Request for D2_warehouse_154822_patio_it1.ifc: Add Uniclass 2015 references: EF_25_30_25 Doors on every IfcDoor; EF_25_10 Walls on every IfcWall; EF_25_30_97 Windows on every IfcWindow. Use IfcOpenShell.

First a look at what the model holds.

```python
import ifcopenshell

model = ifcopenshell.open("D2_warehouse_154822_patio_it1.ifc")
print(model.schema)
print("classifications:", [c.Name for c in model.by_type("IfcClassification")])
for ifc_class in ("IfcDoor", "IfcRoof", "IfcStair", "IfcWall", "IfcWindow"):
    print(ifc_class, len(model.by_type(ifc_class)))
```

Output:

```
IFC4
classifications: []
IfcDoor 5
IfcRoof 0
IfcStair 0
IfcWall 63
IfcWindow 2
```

```python
import ifcopenshell
import ifcopenshell.api.classification

model = ifcopenshell.open("D2_warehouse_154822_patio_it1.ifc")

system = ifcopenshell.api.classification.add_classification(model, classification="Uniclass 2015")

codes = {
    "IfcDoor": ("EF_25_30_25", "Doors"),
    "IfcWall": ("EF_25_10", "Walls"),
    "IfcWindow": ("EF_25_30_97", "Windows"),
}
for ifc_class, (code, name) in codes.items():
    products = model.by_type(ifc_class)
    ifcopenshell.api.classification.add_reference(
        model, products=products, classification=system, identification=code, name=name
    )
    print(code, len(products))

model.write("D2_warehouse_154822_patio_it1_rev.ifc")
```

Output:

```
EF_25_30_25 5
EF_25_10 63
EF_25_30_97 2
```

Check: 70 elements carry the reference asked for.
